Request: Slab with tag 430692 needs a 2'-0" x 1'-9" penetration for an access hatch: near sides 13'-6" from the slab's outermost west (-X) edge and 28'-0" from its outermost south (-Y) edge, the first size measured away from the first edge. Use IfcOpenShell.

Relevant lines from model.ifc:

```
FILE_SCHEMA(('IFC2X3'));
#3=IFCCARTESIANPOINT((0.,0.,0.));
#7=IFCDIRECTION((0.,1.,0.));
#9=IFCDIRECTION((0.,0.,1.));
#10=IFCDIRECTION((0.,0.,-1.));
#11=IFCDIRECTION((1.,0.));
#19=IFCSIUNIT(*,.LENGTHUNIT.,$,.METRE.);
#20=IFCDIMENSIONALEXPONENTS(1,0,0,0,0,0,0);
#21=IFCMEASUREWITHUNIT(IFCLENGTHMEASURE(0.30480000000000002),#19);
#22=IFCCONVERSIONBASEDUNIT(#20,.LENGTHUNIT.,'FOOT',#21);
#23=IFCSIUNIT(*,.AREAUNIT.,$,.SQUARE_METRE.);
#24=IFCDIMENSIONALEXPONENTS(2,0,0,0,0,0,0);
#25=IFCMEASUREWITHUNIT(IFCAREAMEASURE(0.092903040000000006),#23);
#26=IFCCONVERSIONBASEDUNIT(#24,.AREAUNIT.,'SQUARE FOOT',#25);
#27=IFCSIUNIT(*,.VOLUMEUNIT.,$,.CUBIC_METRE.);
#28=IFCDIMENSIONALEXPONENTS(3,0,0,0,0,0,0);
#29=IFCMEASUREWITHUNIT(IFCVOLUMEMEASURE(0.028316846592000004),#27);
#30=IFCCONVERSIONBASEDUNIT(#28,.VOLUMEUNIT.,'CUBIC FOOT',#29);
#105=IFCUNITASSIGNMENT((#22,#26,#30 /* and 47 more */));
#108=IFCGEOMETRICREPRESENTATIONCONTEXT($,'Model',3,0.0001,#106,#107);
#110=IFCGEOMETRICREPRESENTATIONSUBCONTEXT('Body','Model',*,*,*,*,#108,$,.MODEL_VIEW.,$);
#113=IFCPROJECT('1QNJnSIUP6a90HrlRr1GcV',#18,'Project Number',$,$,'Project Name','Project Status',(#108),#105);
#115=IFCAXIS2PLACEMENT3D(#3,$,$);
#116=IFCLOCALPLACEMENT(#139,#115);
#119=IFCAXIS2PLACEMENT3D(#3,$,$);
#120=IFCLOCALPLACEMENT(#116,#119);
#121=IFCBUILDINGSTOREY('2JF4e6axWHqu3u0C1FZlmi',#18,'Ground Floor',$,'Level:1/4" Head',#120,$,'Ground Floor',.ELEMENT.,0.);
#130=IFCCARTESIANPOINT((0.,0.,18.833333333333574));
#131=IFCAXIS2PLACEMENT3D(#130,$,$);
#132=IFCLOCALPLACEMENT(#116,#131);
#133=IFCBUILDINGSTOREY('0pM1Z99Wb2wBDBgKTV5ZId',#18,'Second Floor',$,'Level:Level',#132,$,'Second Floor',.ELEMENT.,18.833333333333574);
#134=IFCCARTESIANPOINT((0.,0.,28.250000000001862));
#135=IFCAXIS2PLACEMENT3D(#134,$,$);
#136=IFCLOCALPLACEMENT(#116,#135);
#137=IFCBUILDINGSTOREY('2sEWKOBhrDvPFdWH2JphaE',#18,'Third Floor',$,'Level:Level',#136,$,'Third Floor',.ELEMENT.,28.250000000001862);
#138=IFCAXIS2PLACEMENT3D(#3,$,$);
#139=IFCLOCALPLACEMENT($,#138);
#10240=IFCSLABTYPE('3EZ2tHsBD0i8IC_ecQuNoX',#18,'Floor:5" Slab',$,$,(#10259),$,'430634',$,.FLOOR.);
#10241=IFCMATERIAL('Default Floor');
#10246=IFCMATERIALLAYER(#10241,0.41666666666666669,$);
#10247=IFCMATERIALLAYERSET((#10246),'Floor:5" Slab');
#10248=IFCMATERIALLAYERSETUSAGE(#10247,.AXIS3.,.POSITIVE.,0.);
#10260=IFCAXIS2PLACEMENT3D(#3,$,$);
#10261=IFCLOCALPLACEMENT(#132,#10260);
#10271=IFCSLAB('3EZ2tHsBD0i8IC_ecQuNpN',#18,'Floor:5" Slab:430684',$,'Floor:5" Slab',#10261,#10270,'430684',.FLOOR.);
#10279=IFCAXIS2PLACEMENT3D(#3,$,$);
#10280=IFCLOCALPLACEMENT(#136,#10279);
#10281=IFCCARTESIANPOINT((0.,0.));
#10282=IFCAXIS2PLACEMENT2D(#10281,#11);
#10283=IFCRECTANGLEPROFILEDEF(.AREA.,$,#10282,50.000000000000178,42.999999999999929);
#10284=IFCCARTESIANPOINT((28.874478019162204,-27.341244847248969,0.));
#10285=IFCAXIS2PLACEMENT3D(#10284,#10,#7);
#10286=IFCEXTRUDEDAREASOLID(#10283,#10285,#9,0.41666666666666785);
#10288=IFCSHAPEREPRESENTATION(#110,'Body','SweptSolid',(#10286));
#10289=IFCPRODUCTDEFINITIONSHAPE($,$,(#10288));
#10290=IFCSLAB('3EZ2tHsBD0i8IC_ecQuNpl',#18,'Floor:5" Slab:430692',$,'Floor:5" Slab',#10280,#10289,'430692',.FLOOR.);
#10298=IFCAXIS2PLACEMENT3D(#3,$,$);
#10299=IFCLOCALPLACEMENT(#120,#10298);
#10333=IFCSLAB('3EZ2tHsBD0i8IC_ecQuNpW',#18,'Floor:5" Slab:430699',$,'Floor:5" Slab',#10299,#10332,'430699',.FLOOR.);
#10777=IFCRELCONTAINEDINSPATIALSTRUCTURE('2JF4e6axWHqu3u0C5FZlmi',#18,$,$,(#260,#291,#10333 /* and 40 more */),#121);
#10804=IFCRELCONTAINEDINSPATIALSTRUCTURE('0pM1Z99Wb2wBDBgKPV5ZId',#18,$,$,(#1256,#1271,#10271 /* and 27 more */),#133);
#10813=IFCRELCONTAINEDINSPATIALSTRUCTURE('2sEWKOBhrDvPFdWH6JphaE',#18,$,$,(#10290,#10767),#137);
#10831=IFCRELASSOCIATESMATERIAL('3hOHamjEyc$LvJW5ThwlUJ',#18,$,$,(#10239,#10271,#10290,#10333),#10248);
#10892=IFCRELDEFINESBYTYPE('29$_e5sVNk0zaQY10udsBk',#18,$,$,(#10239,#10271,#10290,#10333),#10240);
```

```python
import numpy as np
import ifcopenshell
import ifcopenshell.api.feature
import ifcopenshell.api.geometry
import ifcopenshell.api.root
import ifcopenshell.geom
import ifcopenshell.util.placement
import ifcopenshell.util.representation
import ifcopenshell.util.shape
import ifcopenshell.util.unit

model = ifcopenshell.open("model.ifc")
unit_scale = ifcopenshell.util.unit.calculate_unit_scale(model)
settings = ifcopenshell.geom.settings()


def volume(element):
    """Net volume in cubic metres, openings subtracted."""
    shape = ifcopenshell.geom.create_shape(settings, element)
    return ifcopenshell.util.shape.get_volume(shape.geometry)


slab = model.by_id(10290)
before = volume(slab)

# Extent in the slab's own axes, in metres. The edges named are its -X and -Y sides.
slab_shape = ifcopenshell.geom.create_shape(settings, slab)
vertices = ifcopenshell.util.shape.get_vertices(slab_shape.geometry)
x_min, y_min, bottom = vertices.min(axis=0)
top = vertices[:, 2].max()

opening = ifcopenshell.api.root.create_entity(model, ifc_class="IfcOpeningElement", name="Access hatch opening")
context = ifcopenshell.util.representation.get_context(model, "Model", "Body", "MODEL_VIEW")
width, depth = 0.6096, 0.5334
outline = [(0.0, 0.0), (width, 0.0), (width, depth), (0.0, depth), (0.0, 0.0)]
# Overshoot both faces by 50 mm so the cut is clean.
shape = ifcopenshell.api.geometry.add_slab_representation(
    model, context=context, depth=top - bottom + 0.1, polyline=outline
)
ifcopenshell.api.geometry.assign_representation(model, product=opening, representation=shape)

matrix = ifcopenshell.util.placement.get_local_placement(slab.ObjectPlacement)
matrix[:, 3] = matrix @ np.append(np.array([x_min + 4.1148, y_min + 8.5344, bottom - 0.05]) / unit_scale, 1.0)
ifcopenshell.api.geometry.edit_object_placement(model, product=opening, matrix=matrix, is_si=False)
ifcopenshell.api.feature.add_feature(model, feature=opening, element=slab)

after = volume(slab)

print(f"slab volume {before:.3f} -> {after:.3f} m3")

model.write("model_rev.ifc")
```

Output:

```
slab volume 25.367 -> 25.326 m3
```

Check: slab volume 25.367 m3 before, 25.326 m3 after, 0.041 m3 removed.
